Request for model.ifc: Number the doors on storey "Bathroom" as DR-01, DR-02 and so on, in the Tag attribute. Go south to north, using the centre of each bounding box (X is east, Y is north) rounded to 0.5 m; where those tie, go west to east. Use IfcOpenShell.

First a look at what the model holds.

```python
import ifcopenshell
import ifcopenshell.util.element
import ifcopenshell.util.placement

model = ifcopenshell.open("model.ifc")
print(model.schema)
storey = next(s for s in model.by_type("IfcBuildingStorey") if s.Name == "Bathroom")
doors = [e for e in ifcopenshell.util.element.get_decomposition(storey) if e.is_a("IfcDoor")]
for e in sorted(doors, key=lambda e: e.id()):
    origin = ifcopenshell.util.placement.get_local_placement(e.ObjectPlacement)[:3, 3]
    print(e.id(), e.Tag, e.Name, origin.round(2) + 0.0, sep=" | ")
```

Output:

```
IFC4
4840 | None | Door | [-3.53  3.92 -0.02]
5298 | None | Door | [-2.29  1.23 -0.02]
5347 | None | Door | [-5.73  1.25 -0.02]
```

```python
import ifcopenshell
import ifcopenshell.geom
import ifcopenshell.util.element
import ifcopenshell.util.shape

model = ifcopenshell.open("model.ifc")
settings = ifcopenshell.geom.settings()
settings.set("use-world-coords", True)


def centre(element):
    shape = ifcopenshell.geom.create_shape(settings, element)
    return ifcopenshell.util.shape.get_bbox_centroid(shape.geometry)


storey = next(s for s in model.by_type("IfcBuildingStorey") if s.Name == "Bathroom")
doors = [e for e in ifcopenshell.util.element.get_decomposition(storey) if e.is_a("IfcDoor")]

# Insertion points can sit at a corner or the storey origin, so sort by the geometry (in metres).
centres = {e: centre(e) for e in doors}
doors.sort(key=lambda e: (round(centres[e][1] / 0.5), centres[e][0]))

for i, e in enumerate(doors, start=1):
    number = f"DR-{i:02d}"
    e.Tag = number
    print(e.id(), number)

model.write("model_edited.ifc")
```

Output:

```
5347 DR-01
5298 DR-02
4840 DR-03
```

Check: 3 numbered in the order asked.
